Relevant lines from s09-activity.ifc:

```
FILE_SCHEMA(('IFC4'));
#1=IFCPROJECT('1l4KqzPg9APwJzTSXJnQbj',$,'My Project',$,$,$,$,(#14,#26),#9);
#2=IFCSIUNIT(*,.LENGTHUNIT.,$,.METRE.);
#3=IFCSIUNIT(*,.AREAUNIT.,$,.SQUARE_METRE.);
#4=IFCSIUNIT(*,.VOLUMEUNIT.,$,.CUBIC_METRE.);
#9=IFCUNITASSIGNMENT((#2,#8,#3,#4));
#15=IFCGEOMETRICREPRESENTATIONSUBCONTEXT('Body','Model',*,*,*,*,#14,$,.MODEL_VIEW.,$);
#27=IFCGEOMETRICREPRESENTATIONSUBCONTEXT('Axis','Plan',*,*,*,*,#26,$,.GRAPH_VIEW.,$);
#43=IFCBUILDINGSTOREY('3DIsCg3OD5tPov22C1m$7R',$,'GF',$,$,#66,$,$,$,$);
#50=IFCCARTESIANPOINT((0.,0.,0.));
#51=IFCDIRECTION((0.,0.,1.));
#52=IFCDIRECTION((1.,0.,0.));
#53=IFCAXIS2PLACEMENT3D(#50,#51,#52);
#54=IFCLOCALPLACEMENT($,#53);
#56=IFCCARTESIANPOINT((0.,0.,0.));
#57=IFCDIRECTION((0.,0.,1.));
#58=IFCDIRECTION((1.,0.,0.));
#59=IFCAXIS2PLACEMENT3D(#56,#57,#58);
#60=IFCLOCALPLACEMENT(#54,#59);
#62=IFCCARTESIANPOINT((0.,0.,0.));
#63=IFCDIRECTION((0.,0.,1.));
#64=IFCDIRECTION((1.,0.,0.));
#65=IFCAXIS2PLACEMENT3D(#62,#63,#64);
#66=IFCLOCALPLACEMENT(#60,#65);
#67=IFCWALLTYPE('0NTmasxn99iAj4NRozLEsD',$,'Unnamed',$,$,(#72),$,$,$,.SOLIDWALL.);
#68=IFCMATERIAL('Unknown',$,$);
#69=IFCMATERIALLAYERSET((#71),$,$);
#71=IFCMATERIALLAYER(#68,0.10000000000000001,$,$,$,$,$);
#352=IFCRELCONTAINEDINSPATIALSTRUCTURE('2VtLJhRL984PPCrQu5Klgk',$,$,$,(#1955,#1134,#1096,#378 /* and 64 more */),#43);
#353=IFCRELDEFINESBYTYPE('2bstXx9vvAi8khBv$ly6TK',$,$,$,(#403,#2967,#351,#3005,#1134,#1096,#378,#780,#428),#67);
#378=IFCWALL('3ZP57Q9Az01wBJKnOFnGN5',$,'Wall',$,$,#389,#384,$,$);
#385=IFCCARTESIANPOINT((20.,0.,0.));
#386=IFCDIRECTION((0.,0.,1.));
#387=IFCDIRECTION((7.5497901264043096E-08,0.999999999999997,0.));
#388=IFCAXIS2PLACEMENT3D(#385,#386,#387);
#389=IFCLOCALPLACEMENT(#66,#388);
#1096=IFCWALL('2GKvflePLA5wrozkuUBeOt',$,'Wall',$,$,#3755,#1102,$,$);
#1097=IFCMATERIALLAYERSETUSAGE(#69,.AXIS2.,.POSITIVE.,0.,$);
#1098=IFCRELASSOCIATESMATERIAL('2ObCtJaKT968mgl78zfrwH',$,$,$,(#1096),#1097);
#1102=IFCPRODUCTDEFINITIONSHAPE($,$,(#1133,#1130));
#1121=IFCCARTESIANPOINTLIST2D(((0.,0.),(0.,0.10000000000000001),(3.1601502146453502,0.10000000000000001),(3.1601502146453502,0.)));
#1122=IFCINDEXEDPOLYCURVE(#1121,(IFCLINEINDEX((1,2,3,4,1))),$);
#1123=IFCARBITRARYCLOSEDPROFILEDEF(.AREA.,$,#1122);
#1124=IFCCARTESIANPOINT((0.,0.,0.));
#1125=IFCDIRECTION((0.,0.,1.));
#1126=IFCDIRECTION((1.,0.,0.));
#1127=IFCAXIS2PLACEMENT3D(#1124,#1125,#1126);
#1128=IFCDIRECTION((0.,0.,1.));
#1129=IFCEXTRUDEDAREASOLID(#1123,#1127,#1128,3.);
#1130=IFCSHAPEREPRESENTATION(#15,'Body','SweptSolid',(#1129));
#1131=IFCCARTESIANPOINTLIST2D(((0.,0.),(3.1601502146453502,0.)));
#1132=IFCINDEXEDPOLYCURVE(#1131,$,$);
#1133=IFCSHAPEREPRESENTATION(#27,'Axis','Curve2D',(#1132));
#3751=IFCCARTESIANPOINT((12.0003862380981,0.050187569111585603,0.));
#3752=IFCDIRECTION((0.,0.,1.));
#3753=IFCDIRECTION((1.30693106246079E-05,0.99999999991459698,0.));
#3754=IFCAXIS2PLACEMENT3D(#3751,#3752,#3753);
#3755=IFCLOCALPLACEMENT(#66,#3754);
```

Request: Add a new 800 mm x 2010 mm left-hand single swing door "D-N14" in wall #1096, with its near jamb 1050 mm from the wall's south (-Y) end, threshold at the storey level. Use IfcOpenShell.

```python
import numpy as np
import ifcopenshell
import ifcopenshell.api.feature
import ifcopenshell.api.geometry
import ifcopenshell.api.root
import ifcopenshell.api.spatial
import ifcopenshell.geom
import ifcopenshell.util.element
import ifcopenshell.util.placement
import ifcopenshell.util.representation
import ifcopenshell.util.shape
import ifcopenshell.util.unit

model = ifcopenshell.open("s09-activity.ifc")
unit_scale = ifcopenshell.util.unit.calculate_unit_scale(model)
settings = ifcopenshell.geom.settings()


def volume(element):
    """Net volume in cubic metres, openings subtracted."""
    shape = ifcopenshell.geom.create_shape(settings, element)
    return ifcopenshell.util.shape.get_volume(shape.geometry)


wall = model.by_guid("2GKvflePLA5wrozkuUBeOt")
storey = ifcopenshell.util.element.get_container(wall, ifc_class="IfcBuildingStorey")
context = ifcopenshell.util.representation.get_context(model, "Model", "Body", "MODEL_VIEW")
before = volume(wall)

width, height, from_end, sill = 0.8, 2.01, 1.05, 0.0  # metres

# The wall runs along its own X axis, and the end named is its -X end.
wall_shape = ifcopenshell.geom.create_shape(settings, wall)
x, y, z = ifcopenshell.util.shape.get_vertices(wall_shape.geometry).T
start = x.min() + from_end
face, thickness = float(y.min()), float(y.max() - y.min())
wall_matrix = ifcopenshell.util.placement.get_local_placement(wall.ObjectPlacement)
level = ifcopenshell.util.placement.get_local_placement(storey.ObjectPlacement)[2, 3]


def in_wall(x, y):
    """Placement at x, y metres in the wall's axes, at sill height."""
    matrix = wall_matrix.copy()
    matrix[:, 3] = wall_matrix @ np.array([x / unit_scale, y / unit_scale, 0.0, 1.0])
    matrix[2, 3] = level + sill / unit_scale
    return matrix


# Opening: a box that overshoots both wall faces by 50 mm.
opening = ifcopenshell.api.root.create_entity(model, ifc_class="IfcOpeningElement", predefined_type="OPENING")
box = ifcopenshell.api.geometry.add_wall_representation(
    model, context=context, length=width, height=height, thickness=thickness + 0.1
)
ifcopenshell.api.geometry.assign_representation(model, product=opening, representation=box)
ifcopenshell.api.geometry.edit_object_placement(model, product=opening, matrix=in_wall(start, face - 0.05), is_si=False)
ifcopenshell.api.feature.add_feature(model, feature=opening, element=wall)

door = ifcopenshell.api.root.create_entity(model, ifc_class="IfcDoor", name="D-N14", predefined_type="DOOR")
door.OverallWidth, door.OverallHeight = width / unit_scale, height / unit_scale
door.OperationType = "SINGLE_SWING_LEFT"
body = ifcopenshell.api.geometry.add_door_representation(
    model,
    context=context,
    overall_width=door.OverallWidth,
    overall_height=door.OverallHeight,
    operation_type="SINGLE_SWING_LEFT",
    lining_properties={"LiningDepth": thickness / unit_scale, "ThresholdDepth": thickness / unit_scale},
)
ifcopenshell.api.geometry.assign_representation(model, product=door, representation=body)
ifcopenshell.api.spatial.assign_container(model, products=[door], relating_structure=storey)
ifcopenshell.api.feature.add_filling(model, opening=opening, element=door)

# The lining spans the wall, so the door starts at the wall face.
ifcopenshell.api.geometry.edit_object_placement(model, product=door, matrix=in_wall(start, face), is_si=False)

after = volume(wall)

print(f"wall volume {before:.3f} -> {after:.3f} m3")

model.write("s09-activity_edited.ifc")
```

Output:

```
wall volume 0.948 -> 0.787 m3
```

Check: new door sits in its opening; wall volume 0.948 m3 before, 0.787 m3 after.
